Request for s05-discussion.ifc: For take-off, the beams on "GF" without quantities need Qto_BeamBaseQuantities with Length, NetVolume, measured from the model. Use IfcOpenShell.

First a look at what the model holds.

```python
import ifcopenshell
import ifcopenshell.util.element
import ifcopenshell.util.unit

model = ifcopenshell.open("s05-discussion.ifc")
print(model.schema)
for unit_type in ("LENGTHUNIT", "AREAUNIT", "VOLUMEUNIT"):
    print(unit_type, ifcopenshell.util.unit.calculate_unit_scale(model, unit_type))
storey = next(s for s in model.by_type("IfcBuildingStorey") if s.Name == "GF")
beams = [e for e in ifcopenshell.util.element.get_decomposition(storey) if e.is_a("IfcBeam")]
for e in sorted(beams, key=lambda e: e.id()):
    print(e.id(), e.is_a(), e.Name, list(ifcopenshell.util.element.get_psets(e, qtos_only=True)), sep=" | ")
```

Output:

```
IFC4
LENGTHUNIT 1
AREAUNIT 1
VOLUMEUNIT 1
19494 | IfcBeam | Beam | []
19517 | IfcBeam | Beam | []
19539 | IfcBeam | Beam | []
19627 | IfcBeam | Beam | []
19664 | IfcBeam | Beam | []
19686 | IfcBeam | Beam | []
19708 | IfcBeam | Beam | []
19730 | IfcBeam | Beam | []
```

```python
import ifcopenshell
import ifcopenshell.api.pset
import ifcopenshell.geom
import ifcopenshell.util.element
import ifcopenshell.util.shape
import ifcopenshell.util.unit

model = ifcopenshell.open("s05-discussion.ifc")
unit_scale = ifcopenshell.util.unit.calculate_unit_scale(model)
volume_scale = ifcopenshell.util.unit.calculate_unit_scale(model, "VOLUMEUNIT")
settings = ifcopenshell.geom.settings()

storey = next(s for s in model.by_type("IfcBuildingStorey") if s.Name == "GF")
beams = [e for e in ifcopenshell.util.element.get_decomposition(storey) if e.is_a("IfcBeam")]

for e in sorted(beams, key=lambda e: e.id()):
    if ifcopenshell.util.element.get_psets(e, qtos_only=True, should_inherit=False):
        continue
    # Geometry comes back in metres, in the element's own axes.
    shape = ifcopenshell.geom.create_shape(settings, e)
    values = {
        "Length": ifcopenshell.util.shape.get_max_xyz(shape.geometry) / unit_scale,
        "NetVolume": ifcopenshell.util.shape.get_volume(shape.geometry) / volume_scale,
    }
    qto = ifcopenshell.api.pset.add_qto(model, product=e, name="Qto_BeamBaseQuantities")
    ifcopenshell.api.pset.edit_qto(model, qto=qto, properties=values)
    print(e.id(), {k: round(v, 3) for k, v in values.items()})

model.write("s05-discussion-out.ifc")
```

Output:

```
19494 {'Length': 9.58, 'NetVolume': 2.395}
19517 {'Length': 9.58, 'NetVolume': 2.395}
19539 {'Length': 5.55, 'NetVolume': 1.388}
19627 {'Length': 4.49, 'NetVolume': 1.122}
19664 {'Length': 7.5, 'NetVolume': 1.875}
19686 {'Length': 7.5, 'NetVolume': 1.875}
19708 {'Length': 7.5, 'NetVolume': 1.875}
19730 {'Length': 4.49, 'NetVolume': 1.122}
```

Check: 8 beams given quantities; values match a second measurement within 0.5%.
